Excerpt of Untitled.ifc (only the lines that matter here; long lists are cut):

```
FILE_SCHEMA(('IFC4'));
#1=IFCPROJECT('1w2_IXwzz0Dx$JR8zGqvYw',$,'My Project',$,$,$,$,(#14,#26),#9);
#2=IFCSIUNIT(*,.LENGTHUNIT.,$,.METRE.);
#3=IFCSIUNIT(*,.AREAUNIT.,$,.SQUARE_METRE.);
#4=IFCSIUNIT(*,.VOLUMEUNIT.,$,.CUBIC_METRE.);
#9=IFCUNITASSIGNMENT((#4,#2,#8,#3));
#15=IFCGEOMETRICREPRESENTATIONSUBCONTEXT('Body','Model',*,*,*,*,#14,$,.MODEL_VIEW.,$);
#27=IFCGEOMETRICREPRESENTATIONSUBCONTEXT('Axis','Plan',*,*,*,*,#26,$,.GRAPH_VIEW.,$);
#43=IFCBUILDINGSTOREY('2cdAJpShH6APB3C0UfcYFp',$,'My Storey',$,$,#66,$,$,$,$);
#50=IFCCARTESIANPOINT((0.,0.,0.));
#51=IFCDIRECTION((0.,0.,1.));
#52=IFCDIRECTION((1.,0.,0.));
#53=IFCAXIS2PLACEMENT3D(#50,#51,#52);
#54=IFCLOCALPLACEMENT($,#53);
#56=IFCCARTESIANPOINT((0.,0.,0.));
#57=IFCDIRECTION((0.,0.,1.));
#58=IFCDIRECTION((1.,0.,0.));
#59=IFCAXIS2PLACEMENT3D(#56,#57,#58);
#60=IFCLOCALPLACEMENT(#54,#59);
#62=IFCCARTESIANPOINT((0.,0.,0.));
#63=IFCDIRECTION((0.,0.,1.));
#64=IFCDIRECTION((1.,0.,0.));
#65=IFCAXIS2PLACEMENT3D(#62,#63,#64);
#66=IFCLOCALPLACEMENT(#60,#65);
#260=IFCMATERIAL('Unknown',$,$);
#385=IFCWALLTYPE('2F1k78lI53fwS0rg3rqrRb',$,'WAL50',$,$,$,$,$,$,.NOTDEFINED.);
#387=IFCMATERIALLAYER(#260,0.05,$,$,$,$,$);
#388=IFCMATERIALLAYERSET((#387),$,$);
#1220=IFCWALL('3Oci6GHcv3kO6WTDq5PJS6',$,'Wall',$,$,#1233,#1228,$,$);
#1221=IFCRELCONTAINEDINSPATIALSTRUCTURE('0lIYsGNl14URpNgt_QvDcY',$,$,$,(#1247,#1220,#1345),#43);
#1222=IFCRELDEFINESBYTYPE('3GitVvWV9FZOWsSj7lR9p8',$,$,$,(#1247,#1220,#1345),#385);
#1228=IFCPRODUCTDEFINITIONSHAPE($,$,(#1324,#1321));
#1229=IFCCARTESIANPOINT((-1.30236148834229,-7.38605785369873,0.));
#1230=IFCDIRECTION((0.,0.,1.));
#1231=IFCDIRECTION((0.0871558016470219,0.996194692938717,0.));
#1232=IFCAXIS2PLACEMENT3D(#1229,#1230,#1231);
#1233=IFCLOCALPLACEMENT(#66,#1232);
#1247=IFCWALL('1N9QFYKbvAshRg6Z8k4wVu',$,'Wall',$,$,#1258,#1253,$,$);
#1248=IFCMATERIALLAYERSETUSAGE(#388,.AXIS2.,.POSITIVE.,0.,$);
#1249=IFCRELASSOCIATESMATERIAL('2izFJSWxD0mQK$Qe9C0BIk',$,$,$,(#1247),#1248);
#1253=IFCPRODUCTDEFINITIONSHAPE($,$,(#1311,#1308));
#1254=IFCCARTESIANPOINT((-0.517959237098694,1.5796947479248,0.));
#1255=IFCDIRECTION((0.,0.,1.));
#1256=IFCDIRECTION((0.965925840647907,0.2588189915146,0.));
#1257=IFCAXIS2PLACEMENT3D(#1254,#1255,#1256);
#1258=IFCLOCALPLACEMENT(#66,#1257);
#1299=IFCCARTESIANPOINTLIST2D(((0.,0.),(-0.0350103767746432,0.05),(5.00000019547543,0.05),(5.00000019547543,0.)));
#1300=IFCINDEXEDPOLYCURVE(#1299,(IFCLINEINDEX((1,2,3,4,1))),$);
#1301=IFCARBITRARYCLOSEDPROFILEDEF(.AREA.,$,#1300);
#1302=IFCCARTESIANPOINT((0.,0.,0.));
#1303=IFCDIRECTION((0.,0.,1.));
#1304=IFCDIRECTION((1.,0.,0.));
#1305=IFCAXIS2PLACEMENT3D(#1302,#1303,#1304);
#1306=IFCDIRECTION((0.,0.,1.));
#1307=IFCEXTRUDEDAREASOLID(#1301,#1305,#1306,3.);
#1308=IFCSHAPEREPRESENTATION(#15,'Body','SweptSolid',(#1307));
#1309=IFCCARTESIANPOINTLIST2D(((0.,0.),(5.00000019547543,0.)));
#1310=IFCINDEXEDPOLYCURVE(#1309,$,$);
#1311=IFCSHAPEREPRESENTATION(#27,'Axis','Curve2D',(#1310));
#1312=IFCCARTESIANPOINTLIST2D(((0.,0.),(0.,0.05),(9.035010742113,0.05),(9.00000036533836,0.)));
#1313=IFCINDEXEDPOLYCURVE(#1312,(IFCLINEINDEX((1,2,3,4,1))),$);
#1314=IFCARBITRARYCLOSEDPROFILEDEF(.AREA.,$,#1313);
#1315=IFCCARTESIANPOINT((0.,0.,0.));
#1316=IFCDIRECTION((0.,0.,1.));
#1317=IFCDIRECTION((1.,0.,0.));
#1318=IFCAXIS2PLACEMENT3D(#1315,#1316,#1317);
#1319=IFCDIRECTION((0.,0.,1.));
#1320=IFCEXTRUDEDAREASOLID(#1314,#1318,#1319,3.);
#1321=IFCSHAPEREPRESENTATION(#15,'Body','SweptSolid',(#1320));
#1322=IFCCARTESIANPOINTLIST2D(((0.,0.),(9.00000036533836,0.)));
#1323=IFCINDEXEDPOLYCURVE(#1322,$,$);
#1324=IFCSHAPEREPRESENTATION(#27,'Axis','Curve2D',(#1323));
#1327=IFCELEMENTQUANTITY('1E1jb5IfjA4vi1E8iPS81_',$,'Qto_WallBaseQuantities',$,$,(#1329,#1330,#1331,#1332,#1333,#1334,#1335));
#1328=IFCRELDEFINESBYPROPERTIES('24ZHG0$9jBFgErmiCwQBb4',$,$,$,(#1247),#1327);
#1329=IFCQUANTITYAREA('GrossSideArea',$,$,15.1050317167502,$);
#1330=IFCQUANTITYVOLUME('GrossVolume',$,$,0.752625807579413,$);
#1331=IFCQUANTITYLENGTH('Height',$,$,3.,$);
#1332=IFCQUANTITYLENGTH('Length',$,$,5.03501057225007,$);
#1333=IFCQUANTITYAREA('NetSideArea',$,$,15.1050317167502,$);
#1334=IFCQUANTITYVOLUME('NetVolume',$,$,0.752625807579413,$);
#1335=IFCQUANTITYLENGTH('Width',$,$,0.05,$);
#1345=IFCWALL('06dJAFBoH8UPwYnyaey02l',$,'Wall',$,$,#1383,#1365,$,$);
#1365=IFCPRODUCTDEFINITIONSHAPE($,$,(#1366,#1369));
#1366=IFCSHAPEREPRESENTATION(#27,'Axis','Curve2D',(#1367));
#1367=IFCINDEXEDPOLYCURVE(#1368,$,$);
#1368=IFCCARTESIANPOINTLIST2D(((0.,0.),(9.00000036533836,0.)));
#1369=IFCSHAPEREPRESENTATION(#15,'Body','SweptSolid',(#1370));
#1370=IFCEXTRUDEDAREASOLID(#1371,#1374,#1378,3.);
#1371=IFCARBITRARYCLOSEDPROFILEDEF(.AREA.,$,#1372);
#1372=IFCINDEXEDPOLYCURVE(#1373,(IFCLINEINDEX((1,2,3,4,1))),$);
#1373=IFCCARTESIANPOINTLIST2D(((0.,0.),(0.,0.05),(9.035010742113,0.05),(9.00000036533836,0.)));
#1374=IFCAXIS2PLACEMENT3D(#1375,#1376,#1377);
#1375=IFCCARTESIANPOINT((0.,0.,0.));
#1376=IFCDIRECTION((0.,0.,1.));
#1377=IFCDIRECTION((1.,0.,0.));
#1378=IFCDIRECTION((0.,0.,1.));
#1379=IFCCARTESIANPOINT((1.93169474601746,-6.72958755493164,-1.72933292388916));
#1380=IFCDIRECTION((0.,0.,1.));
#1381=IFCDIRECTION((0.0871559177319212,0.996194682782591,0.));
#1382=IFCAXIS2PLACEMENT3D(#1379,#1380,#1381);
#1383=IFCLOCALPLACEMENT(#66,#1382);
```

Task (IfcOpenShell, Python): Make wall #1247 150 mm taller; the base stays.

```python
import ifcopenshell
import ifcopenshell.api.pset
import ifcopenshell.geom
import ifcopenshell.util.element
import ifcopenshell.util.representation
import ifcopenshell.util.shape
import ifcopenshell.util.unit

model = ifcopenshell.open("Untitled.ifc")
unit_scale = ifcopenshell.util.unit.calculate_unit_scale(model)
area_scale = ifcopenshell.util.unit.calculate_unit_scale(model, "AREAUNIT")
volume_scale = ifcopenshell.util.unit.calculate_unit_scale(model, "VOLUMEUNIT")
settings = ifcopenshell.geom.settings()


def volume(element):
    """Net volume in cubic metres, openings subtracted."""
    shape = ifcopenshell.geom.create_shape(settings, element)
    return ifcopenshell.util.shape.get_volume(shape.geometry)


wall = model.by_guid("1N9QFYKbvAshRg6Z8k4wVu")
before = volume(wall)

body = ifcopenshell.util.representation.get_representation(wall, "Model", "Body")
solid = body.Items[0]
old_height = solid.Depth
solid.Depth += 0.15
after = volume(wall)
thickness = 0.05  # wall thickness in metres

# Update the stored height, areas and volumes.
qto = model.by_id(ifcopenshell.util.element.get_pset(wall, "Qto_WallBaseQuantities", should_inherit=False)["id"])
ifcopenshell.api.pset.edit_qto(model, qto=qto, properties={
    "GrossSideArea": ifcopenshell.util.element.get_pset(wall, "Qto_WallBaseQuantities", "GrossSideArea") * solid.Depth / old_height,
    "GrossVolume": ifcopenshell.util.element.get_pset(wall, "Qto_WallBaseQuantities", "GrossVolume") * solid.Depth / old_height,
    "Height": solid.Depth,
    "NetSideArea": after / thickness / area_scale,
    "NetVolume": after / volume_scale,
})

print(f"height {old_height:g} -> {solid.Depth:g}, volume {before:.3f} -> {after:.3f} m3")

model.write("Untitled_edited.ifc")
```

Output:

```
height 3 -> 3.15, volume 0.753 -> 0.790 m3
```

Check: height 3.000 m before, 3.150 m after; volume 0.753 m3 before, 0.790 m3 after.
